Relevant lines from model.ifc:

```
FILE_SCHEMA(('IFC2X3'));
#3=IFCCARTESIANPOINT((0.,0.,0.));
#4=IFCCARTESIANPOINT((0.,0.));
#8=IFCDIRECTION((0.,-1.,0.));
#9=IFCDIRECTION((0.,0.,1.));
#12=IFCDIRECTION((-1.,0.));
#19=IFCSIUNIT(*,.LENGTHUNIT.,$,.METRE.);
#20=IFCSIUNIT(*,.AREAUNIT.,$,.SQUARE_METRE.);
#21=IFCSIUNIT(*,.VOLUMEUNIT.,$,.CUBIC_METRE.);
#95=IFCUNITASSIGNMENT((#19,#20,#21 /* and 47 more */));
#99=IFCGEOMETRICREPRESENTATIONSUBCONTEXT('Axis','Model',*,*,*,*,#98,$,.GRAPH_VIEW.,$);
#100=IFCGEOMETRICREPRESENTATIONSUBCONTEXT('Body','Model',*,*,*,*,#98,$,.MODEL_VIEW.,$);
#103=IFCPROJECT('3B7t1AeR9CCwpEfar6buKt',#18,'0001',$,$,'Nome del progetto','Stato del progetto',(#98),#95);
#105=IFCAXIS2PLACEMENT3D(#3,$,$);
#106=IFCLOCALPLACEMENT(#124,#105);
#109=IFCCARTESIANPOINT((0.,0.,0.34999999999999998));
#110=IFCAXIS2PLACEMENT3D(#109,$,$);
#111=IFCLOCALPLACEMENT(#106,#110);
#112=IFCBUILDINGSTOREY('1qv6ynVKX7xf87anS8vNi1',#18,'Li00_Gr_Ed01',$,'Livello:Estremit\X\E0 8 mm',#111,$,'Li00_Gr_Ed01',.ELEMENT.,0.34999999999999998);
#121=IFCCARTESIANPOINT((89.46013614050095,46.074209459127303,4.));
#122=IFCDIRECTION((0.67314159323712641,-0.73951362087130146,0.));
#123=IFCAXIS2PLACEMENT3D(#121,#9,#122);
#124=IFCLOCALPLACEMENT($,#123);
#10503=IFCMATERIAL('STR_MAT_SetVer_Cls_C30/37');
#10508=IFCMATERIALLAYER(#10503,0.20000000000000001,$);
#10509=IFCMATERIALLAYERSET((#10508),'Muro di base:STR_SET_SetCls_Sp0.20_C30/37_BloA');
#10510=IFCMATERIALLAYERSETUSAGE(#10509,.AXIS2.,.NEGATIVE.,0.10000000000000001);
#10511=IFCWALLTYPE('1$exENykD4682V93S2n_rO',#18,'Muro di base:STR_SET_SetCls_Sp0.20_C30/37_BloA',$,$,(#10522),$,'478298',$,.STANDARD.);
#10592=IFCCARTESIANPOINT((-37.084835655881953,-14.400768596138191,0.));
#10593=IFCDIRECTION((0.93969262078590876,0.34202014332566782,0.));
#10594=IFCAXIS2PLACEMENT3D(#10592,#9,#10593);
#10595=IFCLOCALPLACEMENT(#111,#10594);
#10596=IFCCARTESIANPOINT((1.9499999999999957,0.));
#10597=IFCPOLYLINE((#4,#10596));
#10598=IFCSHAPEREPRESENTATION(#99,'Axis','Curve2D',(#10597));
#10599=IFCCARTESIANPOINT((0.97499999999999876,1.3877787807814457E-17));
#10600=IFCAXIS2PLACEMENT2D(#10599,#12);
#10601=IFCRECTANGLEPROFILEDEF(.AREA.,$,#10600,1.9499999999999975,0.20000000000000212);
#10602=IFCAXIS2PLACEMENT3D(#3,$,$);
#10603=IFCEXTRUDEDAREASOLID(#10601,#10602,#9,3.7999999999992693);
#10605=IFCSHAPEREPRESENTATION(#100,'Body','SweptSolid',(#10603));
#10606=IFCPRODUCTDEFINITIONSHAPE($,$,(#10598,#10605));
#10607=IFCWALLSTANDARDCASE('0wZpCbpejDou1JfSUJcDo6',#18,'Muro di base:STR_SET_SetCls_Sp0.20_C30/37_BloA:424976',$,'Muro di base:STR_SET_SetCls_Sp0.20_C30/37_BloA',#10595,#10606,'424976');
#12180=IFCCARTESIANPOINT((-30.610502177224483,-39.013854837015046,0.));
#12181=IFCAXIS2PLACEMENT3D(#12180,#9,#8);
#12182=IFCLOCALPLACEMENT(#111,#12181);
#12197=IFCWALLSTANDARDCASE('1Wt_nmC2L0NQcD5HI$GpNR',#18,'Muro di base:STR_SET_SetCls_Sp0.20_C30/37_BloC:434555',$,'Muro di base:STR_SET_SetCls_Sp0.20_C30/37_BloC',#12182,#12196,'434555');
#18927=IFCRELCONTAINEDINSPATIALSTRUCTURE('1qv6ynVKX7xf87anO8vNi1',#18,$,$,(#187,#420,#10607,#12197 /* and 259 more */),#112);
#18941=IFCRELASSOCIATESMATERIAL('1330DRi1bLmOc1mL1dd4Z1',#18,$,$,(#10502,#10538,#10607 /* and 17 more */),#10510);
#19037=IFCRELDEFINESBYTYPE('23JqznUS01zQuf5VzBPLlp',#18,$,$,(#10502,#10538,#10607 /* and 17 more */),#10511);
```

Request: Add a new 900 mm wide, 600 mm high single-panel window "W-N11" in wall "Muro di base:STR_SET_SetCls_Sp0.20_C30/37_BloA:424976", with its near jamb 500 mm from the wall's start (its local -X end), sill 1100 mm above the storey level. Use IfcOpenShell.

```python
import numpy as np
import ifcopenshell
import ifcopenshell.api.feature
import ifcopenshell.api.geometry
import ifcopenshell.api.root
import ifcopenshell.api.spatial
import ifcopenshell.api.type
import ifcopenshell.geom
import ifcopenshell.util.element
import ifcopenshell.util.placement
import ifcopenshell.util.representation
import ifcopenshell.util.shape
import ifcopenshell.util.unit

model = ifcopenshell.open("model.ifc")
unit_scale = ifcopenshell.util.unit.calculate_unit_scale(model)
settings = ifcopenshell.geom.settings()


def volume(element):
    """Net volume in cubic metres, openings subtracted."""
    shape = ifcopenshell.geom.create_shape(settings, element)
    return ifcopenshell.util.shape.get_volume(shape.geometry)


wall = model.by_guid("0wZpCbpejDou1JfSUJcDo6")
storey = ifcopenshell.util.element.get_container(wall, ifc_class="IfcBuildingStorey")
context = ifcopenshell.util.representation.get_context(model, "Model", "Body", "MODEL_VIEW")
before = volume(wall)

width, height, from_end, sill = 0.9, 0.6, 0.5, 1.1  # metres

# The wall runs along its own X axis, and the end named is its -X end.
wall_shape = ifcopenshell.geom.create_shape(settings, wall)
x, y, z = ifcopenshell.util.shape.get_vertices(wall_shape.geometry).T
start = x.min() + from_end
face, thickness = float(y.min()), float(y.max() - y.min())
wall_matrix = ifcopenshell.util.placement.get_local_placement(wall.ObjectPlacement)
level = ifcopenshell.util.placement.get_local_placement(storey.ObjectPlacement)[2, 3]


def in_wall(x, y):
    """Placement at x, y metres in the wall's axes, at sill height."""
    matrix = wall_matrix.copy()
    matrix[:, 3] = wall_matrix @ np.array([x / unit_scale, y / unit_scale, 0.0, 1.0])
    matrix[2, 3] = level + sill / unit_scale
    return matrix


# Opening: a box that overshoots both wall faces by 50 mm.
opening = ifcopenshell.api.root.create_entity(model, ifc_class="IfcOpeningElement")
box = ifcopenshell.api.geometry.add_wall_representation(
    model, context=context, length=width, height=height, thickness=thickness + 0.1
)
ifcopenshell.api.geometry.assign_representation(model, product=opening, representation=box)
ifcopenshell.api.geometry.edit_object_placement(model, product=opening, matrix=in_wall(start, face - 0.05), is_si=False)
ifcopenshell.api.feature.add_feature(model, feature=opening, element=wall)

window = ifcopenshell.api.root.create_entity(model, ifc_class="IfcWindow", name="W-N11")
window.OverallWidth, window.OverallHeight = width / unit_scale, height / unit_scale
body = ifcopenshell.api.geometry.add_window_representation(
    model,
    context=context,
    overall_width=window.OverallWidth,
    overall_height=window.OverallHeight,
    partition_type="SINGLE_PANEL",
)
ifcopenshell.api.geometry.assign_representation(model, product=window, representation=body)
ifcopenshell.api.spatial.assign_container(model, products=[window], relating_structure=storey)
fills = ifcopenshell.api.feature.add_filling(model, opening=opening, element=window)
fills.OwnerHistory = window.OwnerHistory  # required in IFC2X3

# IFC2X3 keeps the operation on the window style.
style = ifcopenshell.api.root.create_entity(model, ifc_class="IfcWindowStyle", name="W-N11")
style.OperationType, style.ConstructionType = "SINGLE_PANEL", "NOTDEFINED"
style.ParameterTakesPrecedence = style.Sizeable = False
ifcopenshell.api.type.assign_type(model, related_objects=[window], relating_type=style)

# Centre the window in the wall's thickness.
ifcopenshell.api.geometry.edit_object_placement(model, product=window, matrix=in_wall(start, face), is_si=False)
window_shape = ifcopenshell.geom.create_shape(settings, window)
depth = ifcopenshell.util.shape.get_vertices(window_shape.geometry)[:, 1]
offset = face + thickness / 2 - (depth.min() + depth.max()) / 2
ifcopenshell.api.geometry.edit_object_placement(model, product=window, matrix=in_wall(start, offset), is_si=False)

after = volume(wall)

print(f"wall volume {before:.3f} -> {after:.3f} m3")

model.write("model_edited.ifc")
```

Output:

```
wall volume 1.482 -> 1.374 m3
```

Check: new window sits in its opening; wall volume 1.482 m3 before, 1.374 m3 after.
